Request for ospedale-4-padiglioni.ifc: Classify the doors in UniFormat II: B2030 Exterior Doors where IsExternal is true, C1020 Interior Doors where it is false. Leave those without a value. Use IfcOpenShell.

First a look at what the model holds.

```python
import ifcopenshell
import ifcopenshell.util.element

model = ifcopenshell.open("ospedale-4-padiglioni.ifc")
print(model.schema)
print("classifications:", [c.Name for c in model.by_type("IfcClassification")])
values = [ifcopenshell.util.element.get_pset(e, "Pset_DoorCommon", "IsExternal") for e in model.by_type("IfcDoor")]
for value in (True, False, None):
    print("IsExternal", value, values.count(value))
```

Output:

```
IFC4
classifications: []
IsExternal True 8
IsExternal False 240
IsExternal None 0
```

```python
import ifcopenshell
import ifcopenshell.api.classification
import ifcopenshell.util.element

model = ifcopenshell.open("ospedale-4-padiglioni.ifc")

system = ifcopenshell.api.classification.add_classification(model, classification="UniFormat II")

doors = model.by_type("IfcDoor")
external = {e: ifcopenshell.util.element.get_pset(e, "Pset_DoorCommon", "IsExternal") for e in doors}
for flag, code, name in ((True, "B2030", "Exterior Doors"), (False, "C1020", "Interior Doors")):
    products = [e for e in doors if external[e] is flag]
    ifcopenshell.api.classification.add_reference(
        model, products=products, classification=system, identification=code, name=name
    )
    print(code, len(products))

model.write("ospedale-4-padiglioni_edited.ifc")
```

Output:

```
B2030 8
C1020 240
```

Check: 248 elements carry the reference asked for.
